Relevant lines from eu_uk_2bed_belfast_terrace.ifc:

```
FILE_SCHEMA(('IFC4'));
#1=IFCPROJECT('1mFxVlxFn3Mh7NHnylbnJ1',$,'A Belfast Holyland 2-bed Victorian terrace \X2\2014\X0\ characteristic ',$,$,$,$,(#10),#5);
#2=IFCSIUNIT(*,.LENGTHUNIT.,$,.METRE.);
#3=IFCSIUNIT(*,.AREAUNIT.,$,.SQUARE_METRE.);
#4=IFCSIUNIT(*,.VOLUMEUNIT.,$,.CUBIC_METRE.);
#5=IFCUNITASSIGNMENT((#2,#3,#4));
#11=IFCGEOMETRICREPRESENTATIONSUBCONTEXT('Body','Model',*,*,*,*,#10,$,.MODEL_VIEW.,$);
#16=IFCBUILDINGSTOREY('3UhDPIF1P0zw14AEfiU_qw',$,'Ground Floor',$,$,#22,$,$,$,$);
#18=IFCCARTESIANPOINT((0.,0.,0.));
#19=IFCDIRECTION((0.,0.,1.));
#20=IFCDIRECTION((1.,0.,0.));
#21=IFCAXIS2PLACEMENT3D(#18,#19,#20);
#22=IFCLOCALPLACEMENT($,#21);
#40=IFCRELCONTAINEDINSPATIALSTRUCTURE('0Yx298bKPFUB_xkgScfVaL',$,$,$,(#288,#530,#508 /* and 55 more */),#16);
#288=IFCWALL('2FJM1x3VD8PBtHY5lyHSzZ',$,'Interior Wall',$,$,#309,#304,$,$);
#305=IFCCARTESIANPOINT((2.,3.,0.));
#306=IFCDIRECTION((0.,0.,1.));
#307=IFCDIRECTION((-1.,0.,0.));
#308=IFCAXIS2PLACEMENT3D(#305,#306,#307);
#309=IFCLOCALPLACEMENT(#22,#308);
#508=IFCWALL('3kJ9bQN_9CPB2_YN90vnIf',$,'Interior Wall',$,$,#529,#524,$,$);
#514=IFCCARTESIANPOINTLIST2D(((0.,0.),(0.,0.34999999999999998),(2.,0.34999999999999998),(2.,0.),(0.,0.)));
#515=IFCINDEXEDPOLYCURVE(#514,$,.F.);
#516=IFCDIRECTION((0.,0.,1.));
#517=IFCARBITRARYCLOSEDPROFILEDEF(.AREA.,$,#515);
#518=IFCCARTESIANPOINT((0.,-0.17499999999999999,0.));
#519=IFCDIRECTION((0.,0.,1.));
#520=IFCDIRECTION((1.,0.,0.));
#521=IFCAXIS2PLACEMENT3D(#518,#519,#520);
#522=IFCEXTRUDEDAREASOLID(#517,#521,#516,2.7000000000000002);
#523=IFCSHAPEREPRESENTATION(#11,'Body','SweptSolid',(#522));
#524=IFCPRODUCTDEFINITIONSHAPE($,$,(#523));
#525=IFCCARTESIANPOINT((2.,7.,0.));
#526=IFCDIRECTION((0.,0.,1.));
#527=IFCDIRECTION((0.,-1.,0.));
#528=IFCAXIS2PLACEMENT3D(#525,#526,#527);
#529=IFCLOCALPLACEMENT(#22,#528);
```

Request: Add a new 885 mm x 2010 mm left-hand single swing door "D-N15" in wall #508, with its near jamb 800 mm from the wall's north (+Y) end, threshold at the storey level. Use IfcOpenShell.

```python
import numpy as np
import ifcopenshell
import ifcopenshell.api.feature
import ifcopenshell.api.geometry
import ifcopenshell.api.root
import ifcopenshell.api.spatial
import ifcopenshell.geom
import ifcopenshell.util.element
import ifcopenshell.util.placement
import ifcopenshell.util.representation
import ifcopenshell.util.shape
import ifcopenshell.util.unit

model = ifcopenshell.open("eu_uk_2bed_belfast_terrace.ifc")
unit_scale = ifcopenshell.util.unit.calculate_unit_scale(model)
settings = ifcopenshell.geom.settings()


def volume(element):
    """Net volume in cubic metres, openings subtracted."""
    shape = ifcopenshell.geom.create_shape(settings, element)
    return ifcopenshell.util.shape.get_volume(shape.geometry)


wall = model.by_id(508)
storey = ifcopenshell.util.element.get_container(wall, ifc_class="IfcBuildingStorey")
context = ifcopenshell.util.representation.get_context(model, "Model", "Body", "MODEL_VIEW")
before = volume(wall)

width, height, from_end, sill = 0.885, 2.01, 0.8, 0.0  # metres

# The wall runs along its own X axis, and the end named is its -X end.
wall_shape = ifcopenshell.geom.create_shape(settings, wall)
x, y, z = ifcopenshell.util.shape.get_vertices(wall_shape.geometry).T
start = x.min() + from_end
face, thickness = float(y.min()), float(y.max() - y.min())
wall_matrix = ifcopenshell.util.placement.get_local_placement(wall.ObjectPlacement)
level = ifcopenshell.util.placement.get_local_placement(storey.ObjectPlacement)[2, 3]


def in_wall(x, y):
    """Placement at x, y metres in the wall's axes, at sill height."""
    matrix = wall_matrix.copy()
    matrix[:, 3] = wall_matrix @ np.array([x / unit_scale, y / unit_scale, 0.0, 1.0])
    matrix[2, 3] = level + sill / unit_scale
    return matrix


# Opening: a box that overshoots both wall faces by 50 mm.
opening = ifcopenshell.api.root.create_entity(model, ifc_class="IfcOpeningElement", predefined_type="OPENING")
box = ifcopenshell.api.geometry.add_wall_representation(
    model, context=context, length=width, height=height, thickness=thickness + 0.1
)
ifcopenshell.api.geometry.assign_representation(model, product=opening, representation=box)
ifcopenshell.api.geometry.edit_object_placement(model, product=opening, matrix=in_wall(start, face - 0.05), is_si=False)
ifcopenshell.api.feature.add_feature(model, feature=opening, element=wall)

door = ifcopenshell.api.root.create_entity(model, ifc_class="IfcDoor", name="D-N15", predefined_type="DOOR")
door.OverallWidth, door.OverallHeight = width / unit_scale, height / unit_scale
door.OperationType = "SINGLE_SWING_LEFT"
body = ifcopenshell.api.geometry.add_door_representation(
    model,
    context=context,
    overall_width=door.OverallWidth,
    overall_height=door.OverallHeight,
    operation_type="SINGLE_SWING_LEFT",
    lining_properties={"LiningDepth": thickness / unit_scale, "ThresholdDepth": thickness / unit_scale},
)
ifcopenshell.api.geometry.assign_representation(model, product=door, representation=body)
ifcopenshell.api.spatial.assign_container(model, products=[door], relating_structure=storey)
ifcopenshell.api.feature.add_filling(model, opening=opening, element=door)

# The lining spans the wall, so the door starts at the wall face.
ifcopenshell.api.geometry.edit_object_placement(model, product=door, matrix=in_wall(start, face), is_si=False)

after = volume(wall)

print(f"wall volume {before:.3f} -> {after:.3f} m3")

model.write("eu_uk_2bed_belfast_terrace_rev.ifc")
```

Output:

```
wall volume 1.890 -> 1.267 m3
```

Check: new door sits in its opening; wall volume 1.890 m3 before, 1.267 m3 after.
